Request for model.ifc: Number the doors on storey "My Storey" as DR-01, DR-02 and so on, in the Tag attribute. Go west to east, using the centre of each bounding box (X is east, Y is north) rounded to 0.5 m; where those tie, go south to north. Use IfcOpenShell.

First a look at what the model holds.

```python
import ifcopenshell
import ifcopenshell.util.element
import ifcopenshell.util.placement

model = ifcopenshell.open("model.ifc")
print(model.schema)
storey = next(s for s in model.by_type("IfcBuildingStorey") if s.Name == "My Storey")
doors = [e for e in ifcopenshell.util.element.get_decomposition(storey) if e.is_a("IfcDoor")]
for e in sorted(doors, key=lambda e: e.id()):
    origin = ifcopenshell.util.placement.get_local_placement(e.ObjectPlacement)[:3, 3]
    print(e.id(), e.Tag, e.Name, origin.round(2) + 0.0, sep=" | ")
```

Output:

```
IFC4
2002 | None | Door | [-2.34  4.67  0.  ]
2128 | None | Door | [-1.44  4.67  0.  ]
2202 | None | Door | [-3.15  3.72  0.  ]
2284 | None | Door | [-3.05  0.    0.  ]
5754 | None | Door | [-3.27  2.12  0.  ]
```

```python
import ifcopenshell
import ifcopenshell.geom
import ifcopenshell.util.element
import ifcopenshell.util.shape

model = ifcopenshell.open("model.ifc")
settings = ifcopenshell.geom.settings()
settings.set("use-world-coords", True)


def centre(element):
    shape = ifcopenshell.geom.create_shape(settings, element)
    return ifcopenshell.util.shape.get_bbox_centroid(shape.geometry)


storey = next(s for s in model.by_type("IfcBuildingStorey") if s.Name == "My Storey")
doors = [e for e in ifcopenshell.util.element.get_decomposition(storey) if e.is_a("IfcDoor")]

# Insertion points can sit at a corner or the storey origin, so sort by the geometry (in metres).
centres = {e: centre(e) for e in doors}
doors.sort(key=lambda e: (round(centres[e][0] / 0.5), centres[e][1]))

for i, e in enumerate(doors, start=1):
    number = f"DR-{i:02d}"
    e.Tag = number
    print(e.id(), number)

model.write("model_edited.ifc")
```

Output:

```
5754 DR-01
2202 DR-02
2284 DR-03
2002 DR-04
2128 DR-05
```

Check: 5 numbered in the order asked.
